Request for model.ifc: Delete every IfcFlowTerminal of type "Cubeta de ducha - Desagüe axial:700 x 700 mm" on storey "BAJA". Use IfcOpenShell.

First a look at what the model holds.

```python
import ifcopenshell
import ifcopenshell.util.element

model = ifcopenshell.open("model.ifc")
print(model.schema)
storey = next(s for s in model.by_type("IfcBuildingStorey") if s.Name == "BAJA")
terminals = [e for e in ifcopenshell.util.element.get_decomposition(storey) if e.is_a("IfcFlowTerminal")]
seen = {}
for e in terminals:
    element_type = ifcopenshell.util.element.get_type(e)
    name = element_type.Name if element_type not in (None, e) else None
    seen[name] = seen.get(name, 0) + 1
for name, count in sorted(seen.items(), key=str):
    print(count, "x", name)
```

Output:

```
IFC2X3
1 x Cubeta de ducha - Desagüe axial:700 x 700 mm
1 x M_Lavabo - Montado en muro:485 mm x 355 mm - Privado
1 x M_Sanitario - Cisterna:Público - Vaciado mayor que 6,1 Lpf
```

```python
import ifcopenshell
import ifcopenshell.api.root
import ifcopenshell.util.element

model = ifcopenshell.open("model.ifc")

storey = next(s for s in model.by_type("IfcBuildingStorey") if s.Name == "BAJA")
terminals = [e for e in ifcopenshell.util.element.get_decomposition(storey) if e.is_a("IfcFlowTerminal")]
targets = [e for e in terminals if (t := ifcopenshell.util.element.get_type(e)) not in (None, e) and t.Name == "Cubeta de ducha - Desagüe axial:700 x 700 mm"]

for e in targets:
    ifcopenshell.api.root.remove_product(model, product=e)
print(len(targets), "removed")

model.write("model-out.ifc")
```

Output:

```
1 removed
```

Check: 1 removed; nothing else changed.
